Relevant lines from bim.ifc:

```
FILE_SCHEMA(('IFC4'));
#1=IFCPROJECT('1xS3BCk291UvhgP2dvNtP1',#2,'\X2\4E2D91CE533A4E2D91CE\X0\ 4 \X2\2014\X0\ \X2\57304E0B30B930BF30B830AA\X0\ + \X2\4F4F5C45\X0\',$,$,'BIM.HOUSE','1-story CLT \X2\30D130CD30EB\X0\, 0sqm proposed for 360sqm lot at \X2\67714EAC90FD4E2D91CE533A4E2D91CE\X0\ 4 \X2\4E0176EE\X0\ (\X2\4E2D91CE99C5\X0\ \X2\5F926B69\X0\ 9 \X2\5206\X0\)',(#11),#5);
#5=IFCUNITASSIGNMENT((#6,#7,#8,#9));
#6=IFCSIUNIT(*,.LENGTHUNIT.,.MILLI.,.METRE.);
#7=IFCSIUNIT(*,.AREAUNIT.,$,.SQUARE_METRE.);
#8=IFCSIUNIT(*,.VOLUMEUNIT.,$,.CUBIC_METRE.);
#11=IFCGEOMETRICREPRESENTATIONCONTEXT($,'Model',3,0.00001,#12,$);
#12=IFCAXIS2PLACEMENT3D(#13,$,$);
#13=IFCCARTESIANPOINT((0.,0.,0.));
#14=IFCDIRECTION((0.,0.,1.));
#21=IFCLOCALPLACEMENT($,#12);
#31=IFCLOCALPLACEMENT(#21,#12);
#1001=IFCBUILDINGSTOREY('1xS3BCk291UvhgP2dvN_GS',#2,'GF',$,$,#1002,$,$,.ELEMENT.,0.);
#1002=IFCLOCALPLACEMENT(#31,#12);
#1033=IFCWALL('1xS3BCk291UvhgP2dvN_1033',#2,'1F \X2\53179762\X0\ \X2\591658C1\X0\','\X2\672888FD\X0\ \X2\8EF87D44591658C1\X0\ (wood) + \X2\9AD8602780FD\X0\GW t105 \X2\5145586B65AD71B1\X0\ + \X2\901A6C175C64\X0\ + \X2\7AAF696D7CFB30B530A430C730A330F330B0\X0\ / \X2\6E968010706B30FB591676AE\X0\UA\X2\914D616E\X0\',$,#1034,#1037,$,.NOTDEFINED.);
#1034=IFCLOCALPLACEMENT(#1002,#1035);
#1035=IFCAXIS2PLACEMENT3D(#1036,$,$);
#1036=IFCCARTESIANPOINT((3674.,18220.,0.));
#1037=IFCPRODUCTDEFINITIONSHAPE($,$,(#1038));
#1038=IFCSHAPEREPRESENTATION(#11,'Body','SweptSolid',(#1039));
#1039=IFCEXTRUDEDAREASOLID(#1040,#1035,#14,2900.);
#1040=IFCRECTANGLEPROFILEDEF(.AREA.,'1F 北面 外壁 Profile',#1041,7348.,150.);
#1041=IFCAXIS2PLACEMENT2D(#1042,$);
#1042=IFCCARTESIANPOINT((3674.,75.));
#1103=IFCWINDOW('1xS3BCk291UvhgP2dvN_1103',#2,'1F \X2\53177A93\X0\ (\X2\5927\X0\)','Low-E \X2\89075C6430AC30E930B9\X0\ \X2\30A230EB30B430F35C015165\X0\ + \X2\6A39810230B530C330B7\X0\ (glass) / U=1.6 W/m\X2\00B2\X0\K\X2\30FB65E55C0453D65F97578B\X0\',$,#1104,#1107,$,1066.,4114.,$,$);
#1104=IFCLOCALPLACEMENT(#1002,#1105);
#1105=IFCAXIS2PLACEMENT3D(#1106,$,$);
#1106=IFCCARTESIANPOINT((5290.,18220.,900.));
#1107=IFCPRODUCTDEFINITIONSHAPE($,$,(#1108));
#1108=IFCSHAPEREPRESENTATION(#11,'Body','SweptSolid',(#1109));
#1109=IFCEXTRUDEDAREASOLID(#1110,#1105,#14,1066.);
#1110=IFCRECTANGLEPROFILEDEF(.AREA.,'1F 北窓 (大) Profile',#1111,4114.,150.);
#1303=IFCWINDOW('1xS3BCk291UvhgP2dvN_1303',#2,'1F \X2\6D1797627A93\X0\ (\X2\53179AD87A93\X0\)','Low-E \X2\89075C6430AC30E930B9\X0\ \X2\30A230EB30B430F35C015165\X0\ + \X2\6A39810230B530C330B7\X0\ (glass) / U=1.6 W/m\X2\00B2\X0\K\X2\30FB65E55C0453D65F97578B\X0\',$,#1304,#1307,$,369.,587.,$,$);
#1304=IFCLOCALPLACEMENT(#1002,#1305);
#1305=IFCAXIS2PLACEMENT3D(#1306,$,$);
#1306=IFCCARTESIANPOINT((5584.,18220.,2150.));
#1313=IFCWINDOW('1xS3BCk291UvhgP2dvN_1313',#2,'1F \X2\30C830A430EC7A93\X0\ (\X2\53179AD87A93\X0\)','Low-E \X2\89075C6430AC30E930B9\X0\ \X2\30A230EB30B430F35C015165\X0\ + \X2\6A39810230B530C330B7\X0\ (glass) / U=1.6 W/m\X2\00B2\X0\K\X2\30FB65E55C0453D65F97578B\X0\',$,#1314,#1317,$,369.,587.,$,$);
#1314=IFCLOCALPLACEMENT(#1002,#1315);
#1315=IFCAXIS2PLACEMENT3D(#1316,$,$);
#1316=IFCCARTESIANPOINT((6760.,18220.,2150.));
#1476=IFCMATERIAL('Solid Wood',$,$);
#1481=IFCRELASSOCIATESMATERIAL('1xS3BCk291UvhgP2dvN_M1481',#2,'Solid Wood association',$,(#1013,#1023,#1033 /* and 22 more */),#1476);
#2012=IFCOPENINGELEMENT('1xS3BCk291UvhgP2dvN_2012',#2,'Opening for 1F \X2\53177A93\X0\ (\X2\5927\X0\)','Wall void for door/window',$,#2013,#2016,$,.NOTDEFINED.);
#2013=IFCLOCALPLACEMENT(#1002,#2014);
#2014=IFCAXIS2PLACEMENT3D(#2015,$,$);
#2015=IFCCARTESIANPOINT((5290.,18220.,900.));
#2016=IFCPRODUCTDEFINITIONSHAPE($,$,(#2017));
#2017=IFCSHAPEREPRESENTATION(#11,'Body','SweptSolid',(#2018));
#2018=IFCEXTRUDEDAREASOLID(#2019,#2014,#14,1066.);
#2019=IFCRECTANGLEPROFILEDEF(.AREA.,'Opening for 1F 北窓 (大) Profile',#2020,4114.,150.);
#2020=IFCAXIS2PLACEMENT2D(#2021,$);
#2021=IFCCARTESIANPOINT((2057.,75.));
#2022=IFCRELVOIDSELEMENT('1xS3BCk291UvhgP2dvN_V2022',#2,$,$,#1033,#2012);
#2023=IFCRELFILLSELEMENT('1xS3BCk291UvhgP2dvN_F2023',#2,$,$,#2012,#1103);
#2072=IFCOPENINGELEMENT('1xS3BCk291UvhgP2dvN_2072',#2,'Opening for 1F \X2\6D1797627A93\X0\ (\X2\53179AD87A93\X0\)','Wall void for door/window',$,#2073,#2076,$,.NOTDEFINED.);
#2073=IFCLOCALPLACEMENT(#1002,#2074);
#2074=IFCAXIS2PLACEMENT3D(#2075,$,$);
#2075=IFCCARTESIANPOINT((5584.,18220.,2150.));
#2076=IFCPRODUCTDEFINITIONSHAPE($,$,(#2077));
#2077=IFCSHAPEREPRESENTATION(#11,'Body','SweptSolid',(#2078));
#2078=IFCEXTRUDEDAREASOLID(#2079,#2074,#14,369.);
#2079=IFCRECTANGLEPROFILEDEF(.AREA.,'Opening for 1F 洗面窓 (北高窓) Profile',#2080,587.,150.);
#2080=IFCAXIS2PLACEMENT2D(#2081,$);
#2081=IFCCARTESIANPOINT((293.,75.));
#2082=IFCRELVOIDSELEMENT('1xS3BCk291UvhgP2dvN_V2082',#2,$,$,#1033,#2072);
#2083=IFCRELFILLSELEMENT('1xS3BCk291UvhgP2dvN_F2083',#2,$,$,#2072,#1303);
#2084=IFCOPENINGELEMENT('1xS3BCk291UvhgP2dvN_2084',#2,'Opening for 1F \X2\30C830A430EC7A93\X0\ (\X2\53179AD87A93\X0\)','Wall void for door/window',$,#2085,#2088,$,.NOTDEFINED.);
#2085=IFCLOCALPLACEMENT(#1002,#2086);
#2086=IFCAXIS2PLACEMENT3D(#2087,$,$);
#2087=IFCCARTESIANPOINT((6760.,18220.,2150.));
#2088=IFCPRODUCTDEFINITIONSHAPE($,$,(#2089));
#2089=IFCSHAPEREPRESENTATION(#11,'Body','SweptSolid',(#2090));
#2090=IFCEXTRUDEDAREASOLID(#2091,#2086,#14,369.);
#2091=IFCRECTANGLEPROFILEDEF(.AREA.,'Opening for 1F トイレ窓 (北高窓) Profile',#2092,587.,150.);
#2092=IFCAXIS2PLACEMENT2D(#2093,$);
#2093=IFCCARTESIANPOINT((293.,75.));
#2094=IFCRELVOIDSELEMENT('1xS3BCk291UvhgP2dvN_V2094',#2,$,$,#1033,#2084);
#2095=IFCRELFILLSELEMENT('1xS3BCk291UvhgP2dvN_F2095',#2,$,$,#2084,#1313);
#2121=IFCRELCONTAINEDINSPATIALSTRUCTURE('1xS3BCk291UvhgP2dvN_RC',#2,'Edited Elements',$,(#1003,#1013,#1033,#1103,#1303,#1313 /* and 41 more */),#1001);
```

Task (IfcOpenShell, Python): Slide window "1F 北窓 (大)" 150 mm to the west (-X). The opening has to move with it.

```python
import ifcopenshell
import ifcopenshell.api.geometry
import ifcopenshell.util.placement

model = ifcopenshell.open("bim.ifc")

window = model.by_guid("1xS3BCk291UvhgP2dvN_1103")
opening = window.FillsVoids[0].RelatingOpeningElement
wall = opening.VoidsElements[0].RelatingBuildingElement

wall_matrix = ifcopenshell.util.placement.get_local_placement(wall.ObjectPlacement)
shift = wall_matrix[:3, 0] * -150.0
before = ifcopenshell.util.placement.get_local_placement(window.ObjectPlacement)[:3, 3].copy()

# The window is not placed relative to its opening, so move both.
for product in (opening, window):
    matrix = ifcopenshell.util.placement.get_local_placement(product.ObjectPlacement)
    matrix[:3, 3] += shift
    ifcopenshell.api.geometry.edit_object_placement(model, product=product, matrix=matrix, is_si=False)

after = ifcopenshell.util.placement.get_local_placement(window.ObjectPlacement)[:3, 3]
print("window moved by", (after - before).round(3) + 0.0)

model.write("bim-out.ifc")
```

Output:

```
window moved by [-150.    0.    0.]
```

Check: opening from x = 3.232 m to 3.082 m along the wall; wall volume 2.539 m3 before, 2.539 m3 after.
